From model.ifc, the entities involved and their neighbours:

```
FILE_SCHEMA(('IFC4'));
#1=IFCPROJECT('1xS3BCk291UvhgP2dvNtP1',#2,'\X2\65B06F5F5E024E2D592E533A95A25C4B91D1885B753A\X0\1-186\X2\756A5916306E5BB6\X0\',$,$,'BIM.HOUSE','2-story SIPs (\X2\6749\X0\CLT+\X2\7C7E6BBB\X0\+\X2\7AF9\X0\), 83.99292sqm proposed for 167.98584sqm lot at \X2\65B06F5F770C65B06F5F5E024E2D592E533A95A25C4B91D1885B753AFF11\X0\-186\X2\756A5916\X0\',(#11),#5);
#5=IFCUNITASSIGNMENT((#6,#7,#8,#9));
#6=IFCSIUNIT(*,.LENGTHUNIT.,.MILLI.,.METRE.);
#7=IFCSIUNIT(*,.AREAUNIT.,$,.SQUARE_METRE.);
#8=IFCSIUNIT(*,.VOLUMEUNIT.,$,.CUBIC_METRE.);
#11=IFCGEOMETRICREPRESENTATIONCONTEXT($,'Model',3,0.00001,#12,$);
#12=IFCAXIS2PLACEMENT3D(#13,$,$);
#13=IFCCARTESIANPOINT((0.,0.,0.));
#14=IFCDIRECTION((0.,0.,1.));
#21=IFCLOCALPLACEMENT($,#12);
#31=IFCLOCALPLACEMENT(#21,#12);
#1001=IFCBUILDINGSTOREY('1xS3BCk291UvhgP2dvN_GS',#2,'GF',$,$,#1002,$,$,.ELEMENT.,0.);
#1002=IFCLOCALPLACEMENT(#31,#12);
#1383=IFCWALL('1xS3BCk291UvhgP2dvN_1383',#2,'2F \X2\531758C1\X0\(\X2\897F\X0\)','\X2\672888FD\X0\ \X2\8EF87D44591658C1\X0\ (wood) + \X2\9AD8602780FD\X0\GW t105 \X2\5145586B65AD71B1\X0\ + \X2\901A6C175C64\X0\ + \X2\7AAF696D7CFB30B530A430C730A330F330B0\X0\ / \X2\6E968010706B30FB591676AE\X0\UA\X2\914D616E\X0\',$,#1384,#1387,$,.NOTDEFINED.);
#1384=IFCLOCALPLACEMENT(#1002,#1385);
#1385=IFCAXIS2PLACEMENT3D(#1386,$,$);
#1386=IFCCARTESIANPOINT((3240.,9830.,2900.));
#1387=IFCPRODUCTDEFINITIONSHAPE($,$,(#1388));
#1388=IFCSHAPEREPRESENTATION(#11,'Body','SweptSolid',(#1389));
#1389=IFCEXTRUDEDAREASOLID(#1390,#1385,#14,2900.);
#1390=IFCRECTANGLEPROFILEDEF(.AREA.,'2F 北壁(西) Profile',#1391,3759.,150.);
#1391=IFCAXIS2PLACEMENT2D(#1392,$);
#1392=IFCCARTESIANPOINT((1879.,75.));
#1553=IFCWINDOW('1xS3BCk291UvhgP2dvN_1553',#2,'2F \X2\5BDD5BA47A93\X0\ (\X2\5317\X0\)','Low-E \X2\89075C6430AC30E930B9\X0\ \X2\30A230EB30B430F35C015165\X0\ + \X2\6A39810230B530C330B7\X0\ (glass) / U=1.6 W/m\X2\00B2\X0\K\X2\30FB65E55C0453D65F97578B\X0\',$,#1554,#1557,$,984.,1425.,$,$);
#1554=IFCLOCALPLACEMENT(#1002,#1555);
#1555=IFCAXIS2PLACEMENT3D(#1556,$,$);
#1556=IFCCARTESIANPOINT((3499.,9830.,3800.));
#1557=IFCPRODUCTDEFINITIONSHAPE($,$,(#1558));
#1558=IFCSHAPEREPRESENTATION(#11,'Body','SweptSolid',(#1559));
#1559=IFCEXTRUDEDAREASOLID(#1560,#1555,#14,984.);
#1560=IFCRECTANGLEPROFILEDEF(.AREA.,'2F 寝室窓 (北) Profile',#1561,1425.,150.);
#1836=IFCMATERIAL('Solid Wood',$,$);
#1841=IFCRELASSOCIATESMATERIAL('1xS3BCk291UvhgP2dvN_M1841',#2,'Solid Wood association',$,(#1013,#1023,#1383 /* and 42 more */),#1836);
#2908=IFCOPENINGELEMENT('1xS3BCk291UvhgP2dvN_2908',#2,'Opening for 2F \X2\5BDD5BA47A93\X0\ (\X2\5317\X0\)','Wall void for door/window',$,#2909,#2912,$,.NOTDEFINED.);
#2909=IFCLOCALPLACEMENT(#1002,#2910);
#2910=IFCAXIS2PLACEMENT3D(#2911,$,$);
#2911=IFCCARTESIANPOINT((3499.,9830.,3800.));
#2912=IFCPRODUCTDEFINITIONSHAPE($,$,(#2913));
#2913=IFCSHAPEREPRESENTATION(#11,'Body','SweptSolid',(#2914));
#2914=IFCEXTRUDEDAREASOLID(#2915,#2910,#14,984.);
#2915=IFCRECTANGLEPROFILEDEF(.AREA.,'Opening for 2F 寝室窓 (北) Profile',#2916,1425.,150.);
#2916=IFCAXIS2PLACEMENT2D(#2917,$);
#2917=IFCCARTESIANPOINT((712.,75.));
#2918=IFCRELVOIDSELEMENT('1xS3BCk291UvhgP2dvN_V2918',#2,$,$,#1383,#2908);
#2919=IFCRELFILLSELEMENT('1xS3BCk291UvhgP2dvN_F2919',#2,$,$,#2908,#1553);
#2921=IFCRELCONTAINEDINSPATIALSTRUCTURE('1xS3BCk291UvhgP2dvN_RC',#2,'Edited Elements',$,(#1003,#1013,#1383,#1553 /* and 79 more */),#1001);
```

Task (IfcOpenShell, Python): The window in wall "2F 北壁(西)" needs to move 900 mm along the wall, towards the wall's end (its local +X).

```python
import ifcopenshell
import ifcopenshell.api.geometry
import ifcopenshell.util.placement
import ifcopenshell.util.unit

model = ifcopenshell.open("model.ifc")
unit_scale = ifcopenshell.util.unit.calculate_unit_scale(model)

window = model.by_id(1553)
opening = window.FillsVoids[0].RelatingOpeningElement
wall = opening.VoidsElements[0].RelatingBuildingElement

wall_matrix = ifcopenshell.util.placement.get_local_placement(wall.ObjectPlacement)
shift = wall_matrix[:3, 0] * 0.9 / unit_scale
before = ifcopenshell.util.placement.get_local_placement(window.ObjectPlacement)[:3, 3].copy()

# The window is not placed relative to its opening, so move both.
for product in (opening, window):
    matrix = ifcopenshell.util.placement.get_local_placement(product.ObjectPlacement)
    matrix[:3, 3] += shift
    ifcopenshell.api.geometry.edit_object_placement(model, product=product, matrix=matrix, is_si=False)

after = ifcopenshell.util.placement.get_local_placement(window.ObjectPlacement)[:3, 3]
print("window moved by", (after - before).round(3) + 0.0)

model.write("model_rev.ifc")
```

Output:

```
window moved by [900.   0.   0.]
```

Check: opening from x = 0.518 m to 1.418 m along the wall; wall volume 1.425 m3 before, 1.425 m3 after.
